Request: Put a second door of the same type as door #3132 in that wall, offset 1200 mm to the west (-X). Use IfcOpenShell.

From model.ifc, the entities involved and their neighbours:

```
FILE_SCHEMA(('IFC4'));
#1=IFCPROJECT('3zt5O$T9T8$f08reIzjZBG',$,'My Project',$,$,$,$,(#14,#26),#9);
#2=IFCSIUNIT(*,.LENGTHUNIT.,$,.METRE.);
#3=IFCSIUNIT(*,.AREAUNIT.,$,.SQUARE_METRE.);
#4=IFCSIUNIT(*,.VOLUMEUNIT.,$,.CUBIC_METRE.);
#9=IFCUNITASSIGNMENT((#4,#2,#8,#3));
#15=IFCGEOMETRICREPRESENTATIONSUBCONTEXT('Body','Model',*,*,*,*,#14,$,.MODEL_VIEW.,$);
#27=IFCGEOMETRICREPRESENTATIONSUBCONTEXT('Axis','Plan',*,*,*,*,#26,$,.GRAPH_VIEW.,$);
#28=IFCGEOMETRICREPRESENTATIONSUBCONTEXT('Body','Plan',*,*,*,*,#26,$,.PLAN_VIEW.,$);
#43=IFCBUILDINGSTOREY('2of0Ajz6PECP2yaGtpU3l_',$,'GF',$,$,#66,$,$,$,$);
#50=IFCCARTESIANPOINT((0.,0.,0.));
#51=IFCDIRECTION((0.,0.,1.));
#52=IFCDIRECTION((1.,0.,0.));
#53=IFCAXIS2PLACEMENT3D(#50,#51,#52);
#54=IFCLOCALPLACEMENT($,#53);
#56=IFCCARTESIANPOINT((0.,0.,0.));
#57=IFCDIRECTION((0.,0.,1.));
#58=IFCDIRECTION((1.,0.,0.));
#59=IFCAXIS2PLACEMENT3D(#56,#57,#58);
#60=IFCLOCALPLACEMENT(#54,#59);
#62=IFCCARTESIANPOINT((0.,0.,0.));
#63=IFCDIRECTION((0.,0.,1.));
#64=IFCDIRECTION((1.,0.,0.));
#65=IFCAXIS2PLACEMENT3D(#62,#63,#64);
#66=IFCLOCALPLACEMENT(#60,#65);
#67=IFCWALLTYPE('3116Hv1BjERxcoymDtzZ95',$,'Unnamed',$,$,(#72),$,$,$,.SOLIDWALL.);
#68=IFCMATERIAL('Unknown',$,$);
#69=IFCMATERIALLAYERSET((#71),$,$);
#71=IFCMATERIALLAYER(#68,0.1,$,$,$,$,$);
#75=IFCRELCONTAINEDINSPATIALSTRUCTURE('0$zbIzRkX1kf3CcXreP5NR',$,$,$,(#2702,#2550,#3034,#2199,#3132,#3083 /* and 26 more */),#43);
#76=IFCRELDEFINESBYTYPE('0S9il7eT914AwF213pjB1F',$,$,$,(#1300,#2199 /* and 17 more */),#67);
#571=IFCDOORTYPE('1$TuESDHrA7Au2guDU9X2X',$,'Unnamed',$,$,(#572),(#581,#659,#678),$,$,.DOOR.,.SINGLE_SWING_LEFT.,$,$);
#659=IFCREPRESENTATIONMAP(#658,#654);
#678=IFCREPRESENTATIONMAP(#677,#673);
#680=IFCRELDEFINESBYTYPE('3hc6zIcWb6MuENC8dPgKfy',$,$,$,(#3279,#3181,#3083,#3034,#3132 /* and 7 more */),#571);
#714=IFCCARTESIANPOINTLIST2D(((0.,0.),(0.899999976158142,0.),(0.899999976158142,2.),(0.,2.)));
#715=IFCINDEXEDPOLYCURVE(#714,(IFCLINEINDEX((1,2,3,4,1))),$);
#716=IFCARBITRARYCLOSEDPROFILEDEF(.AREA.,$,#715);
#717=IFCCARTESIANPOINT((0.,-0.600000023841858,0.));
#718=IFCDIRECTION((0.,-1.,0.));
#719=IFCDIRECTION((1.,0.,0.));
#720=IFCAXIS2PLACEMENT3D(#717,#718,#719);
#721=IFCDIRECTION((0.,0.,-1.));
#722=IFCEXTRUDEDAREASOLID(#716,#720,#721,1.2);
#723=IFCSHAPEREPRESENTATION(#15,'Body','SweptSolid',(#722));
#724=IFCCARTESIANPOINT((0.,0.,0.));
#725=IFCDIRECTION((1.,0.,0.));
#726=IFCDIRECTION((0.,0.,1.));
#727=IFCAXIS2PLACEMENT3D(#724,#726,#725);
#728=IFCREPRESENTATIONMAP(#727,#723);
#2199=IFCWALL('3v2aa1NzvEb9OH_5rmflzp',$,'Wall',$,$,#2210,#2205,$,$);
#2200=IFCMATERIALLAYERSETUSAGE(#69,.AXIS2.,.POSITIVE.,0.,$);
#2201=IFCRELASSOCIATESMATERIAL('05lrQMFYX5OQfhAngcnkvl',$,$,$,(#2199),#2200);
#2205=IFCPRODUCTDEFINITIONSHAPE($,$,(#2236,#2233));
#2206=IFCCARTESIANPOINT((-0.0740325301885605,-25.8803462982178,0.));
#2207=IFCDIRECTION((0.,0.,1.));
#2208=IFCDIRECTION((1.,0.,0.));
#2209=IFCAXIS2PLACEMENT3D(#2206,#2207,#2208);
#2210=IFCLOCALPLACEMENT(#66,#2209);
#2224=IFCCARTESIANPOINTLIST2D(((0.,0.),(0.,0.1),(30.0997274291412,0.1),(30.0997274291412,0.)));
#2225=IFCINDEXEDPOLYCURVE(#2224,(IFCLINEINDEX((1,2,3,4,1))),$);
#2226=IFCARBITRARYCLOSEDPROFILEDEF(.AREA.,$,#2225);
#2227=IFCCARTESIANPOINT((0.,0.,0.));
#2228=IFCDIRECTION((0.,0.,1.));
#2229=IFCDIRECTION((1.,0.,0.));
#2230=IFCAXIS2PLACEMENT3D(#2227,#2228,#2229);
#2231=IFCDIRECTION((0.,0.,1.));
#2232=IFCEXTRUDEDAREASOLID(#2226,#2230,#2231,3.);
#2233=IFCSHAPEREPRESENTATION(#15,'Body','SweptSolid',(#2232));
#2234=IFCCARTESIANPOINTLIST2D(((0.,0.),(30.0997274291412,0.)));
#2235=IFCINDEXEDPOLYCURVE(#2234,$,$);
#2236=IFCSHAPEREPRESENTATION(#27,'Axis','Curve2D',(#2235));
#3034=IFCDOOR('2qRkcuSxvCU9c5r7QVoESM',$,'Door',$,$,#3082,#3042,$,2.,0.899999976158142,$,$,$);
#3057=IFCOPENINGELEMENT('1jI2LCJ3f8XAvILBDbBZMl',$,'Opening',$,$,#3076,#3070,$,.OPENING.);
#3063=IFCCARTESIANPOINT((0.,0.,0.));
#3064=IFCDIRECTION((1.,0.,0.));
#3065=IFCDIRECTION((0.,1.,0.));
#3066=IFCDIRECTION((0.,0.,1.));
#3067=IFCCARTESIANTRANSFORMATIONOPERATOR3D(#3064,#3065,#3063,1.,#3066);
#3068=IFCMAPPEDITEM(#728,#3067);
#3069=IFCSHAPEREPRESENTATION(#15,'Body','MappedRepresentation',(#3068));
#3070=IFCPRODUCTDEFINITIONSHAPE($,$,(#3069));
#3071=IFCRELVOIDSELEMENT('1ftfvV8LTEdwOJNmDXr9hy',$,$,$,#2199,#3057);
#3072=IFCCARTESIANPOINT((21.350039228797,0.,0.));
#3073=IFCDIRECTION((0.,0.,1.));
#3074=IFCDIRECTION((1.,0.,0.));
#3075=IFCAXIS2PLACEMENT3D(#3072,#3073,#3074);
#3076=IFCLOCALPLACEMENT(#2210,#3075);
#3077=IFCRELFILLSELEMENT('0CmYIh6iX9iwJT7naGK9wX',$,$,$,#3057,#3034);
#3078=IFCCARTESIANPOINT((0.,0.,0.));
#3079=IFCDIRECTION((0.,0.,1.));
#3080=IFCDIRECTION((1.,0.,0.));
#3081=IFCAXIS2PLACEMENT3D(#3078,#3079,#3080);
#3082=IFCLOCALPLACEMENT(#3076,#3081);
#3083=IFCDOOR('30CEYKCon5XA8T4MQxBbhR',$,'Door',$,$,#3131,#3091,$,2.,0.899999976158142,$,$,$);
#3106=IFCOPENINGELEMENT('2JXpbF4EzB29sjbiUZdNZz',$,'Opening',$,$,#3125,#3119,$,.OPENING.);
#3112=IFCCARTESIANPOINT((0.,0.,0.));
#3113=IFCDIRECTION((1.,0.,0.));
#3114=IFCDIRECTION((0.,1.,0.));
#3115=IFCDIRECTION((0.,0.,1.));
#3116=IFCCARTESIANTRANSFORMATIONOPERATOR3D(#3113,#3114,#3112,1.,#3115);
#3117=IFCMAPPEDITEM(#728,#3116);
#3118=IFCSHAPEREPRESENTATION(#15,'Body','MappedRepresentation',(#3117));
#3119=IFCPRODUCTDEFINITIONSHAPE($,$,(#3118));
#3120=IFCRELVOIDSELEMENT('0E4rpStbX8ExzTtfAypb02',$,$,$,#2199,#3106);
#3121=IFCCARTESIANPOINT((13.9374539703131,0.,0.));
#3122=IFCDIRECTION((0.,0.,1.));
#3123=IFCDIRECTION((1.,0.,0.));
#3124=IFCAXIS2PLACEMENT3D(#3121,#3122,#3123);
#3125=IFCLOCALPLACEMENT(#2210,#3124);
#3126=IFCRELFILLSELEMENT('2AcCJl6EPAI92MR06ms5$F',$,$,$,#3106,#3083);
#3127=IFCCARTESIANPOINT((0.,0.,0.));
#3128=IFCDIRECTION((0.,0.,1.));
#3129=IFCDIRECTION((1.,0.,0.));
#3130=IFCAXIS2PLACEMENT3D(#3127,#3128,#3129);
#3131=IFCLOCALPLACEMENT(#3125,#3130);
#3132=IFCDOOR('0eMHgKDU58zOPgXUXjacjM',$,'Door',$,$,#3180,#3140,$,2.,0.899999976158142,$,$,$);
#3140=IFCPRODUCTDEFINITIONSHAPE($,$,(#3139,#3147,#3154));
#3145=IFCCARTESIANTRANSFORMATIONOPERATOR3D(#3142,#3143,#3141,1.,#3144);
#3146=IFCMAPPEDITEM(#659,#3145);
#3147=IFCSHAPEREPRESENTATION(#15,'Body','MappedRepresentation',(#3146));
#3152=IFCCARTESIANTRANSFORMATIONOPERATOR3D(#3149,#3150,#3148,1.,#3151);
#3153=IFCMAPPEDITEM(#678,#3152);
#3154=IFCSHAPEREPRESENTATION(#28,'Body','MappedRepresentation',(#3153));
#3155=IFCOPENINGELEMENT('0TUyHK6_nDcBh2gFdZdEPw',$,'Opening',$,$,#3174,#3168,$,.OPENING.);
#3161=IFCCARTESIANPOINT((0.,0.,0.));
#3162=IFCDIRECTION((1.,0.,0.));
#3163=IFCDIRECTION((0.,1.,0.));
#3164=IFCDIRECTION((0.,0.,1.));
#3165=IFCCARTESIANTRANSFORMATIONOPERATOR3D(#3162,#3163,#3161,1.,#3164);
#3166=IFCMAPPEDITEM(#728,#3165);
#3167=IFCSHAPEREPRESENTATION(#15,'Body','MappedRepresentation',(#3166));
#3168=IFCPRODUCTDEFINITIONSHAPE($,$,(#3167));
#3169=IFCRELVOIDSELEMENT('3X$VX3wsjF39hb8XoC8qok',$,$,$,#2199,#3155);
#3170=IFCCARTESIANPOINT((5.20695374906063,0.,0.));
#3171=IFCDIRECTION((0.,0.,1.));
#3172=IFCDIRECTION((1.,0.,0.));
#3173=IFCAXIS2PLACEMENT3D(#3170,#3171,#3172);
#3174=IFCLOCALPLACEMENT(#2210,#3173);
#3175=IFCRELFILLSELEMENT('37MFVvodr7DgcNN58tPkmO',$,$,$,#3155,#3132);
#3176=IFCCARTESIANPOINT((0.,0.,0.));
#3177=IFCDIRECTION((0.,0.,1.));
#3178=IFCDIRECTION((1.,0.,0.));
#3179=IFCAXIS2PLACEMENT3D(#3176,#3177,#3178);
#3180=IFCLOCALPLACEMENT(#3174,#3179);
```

```python
import ifcopenshell
import ifcopenshell.api.feature
import ifcopenshell.api.geometry
import ifcopenshell.api.root
import ifcopenshell.geom
import ifcopenshell.util.element
import ifcopenshell.util.placement
import ifcopenshell.util.shape
import ifcopenshell.util.unit

model = ifcopenshell.open("model.ifc")
unit_scale = ifcopenshell.util.unit.calculate_unit_scale(model)
settings = ifcopenshell.geom.settings()


def volume(element):
    """Net volume in cubic metres, openings subtracted."""
    shape = ifcopenshell.geom.create_shape(settings, element)
    return ifcopenshell.util.shape.get_volume(shape.geometry)


door = model.by_guid("0eMHgKDU58zOPgXUXjacjM")
opening = door.FillsVoids[0].RelatingOpeningElement
wall = opening.VoidsElements[0].RelatingBuildingElement
before = volume(wall)
shift = ifcopenshell.util.placement.get_local_placement(wall.ObjectPlacement)[:3, 0] * -1.2 / unit_scale

# copy_class copies the void relationship, type, container and properties, but no geometry.
new_opening = ifcopenshell.api.root.copy_class(model, product=opening)
new_opening.Representation = ifcopenshell.util.element.copy_deep(
    model, opening.Representation, exclude=["IfcGeometricRepresentationContext", "IfcRepresentationMap"]
)
new_door = ifcopenshell.api.root.copy_class(model, product=door)
new_door.Representation = ifcopenshell.util.element.copy_deep(
    model, door.Representation, exclude=["IfcGeometricRepresentationContext", "IfcRepresentationMap"]
)
ifcopenshell.api.feature.add_filling(model, opening=new_opening, element=new_door)

for old, new in ((opening, new_opening), (door, new_door)):
    matrix = ifcopenshell.util.placement.get_local_placement(old.ObjectPlacement)
    matrix[:3, 3] += shift
    ifcopenshell.api.geometry.edit_object_placement(model, product=new, matrix=matrix, is_si=False)

after = volume(wall)

print(f"wall volume {before:.3f} -> {after:.3f} m3")

model.write("model_v2.ifc")
```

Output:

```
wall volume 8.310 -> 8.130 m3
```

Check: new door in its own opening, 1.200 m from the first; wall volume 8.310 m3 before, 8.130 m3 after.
